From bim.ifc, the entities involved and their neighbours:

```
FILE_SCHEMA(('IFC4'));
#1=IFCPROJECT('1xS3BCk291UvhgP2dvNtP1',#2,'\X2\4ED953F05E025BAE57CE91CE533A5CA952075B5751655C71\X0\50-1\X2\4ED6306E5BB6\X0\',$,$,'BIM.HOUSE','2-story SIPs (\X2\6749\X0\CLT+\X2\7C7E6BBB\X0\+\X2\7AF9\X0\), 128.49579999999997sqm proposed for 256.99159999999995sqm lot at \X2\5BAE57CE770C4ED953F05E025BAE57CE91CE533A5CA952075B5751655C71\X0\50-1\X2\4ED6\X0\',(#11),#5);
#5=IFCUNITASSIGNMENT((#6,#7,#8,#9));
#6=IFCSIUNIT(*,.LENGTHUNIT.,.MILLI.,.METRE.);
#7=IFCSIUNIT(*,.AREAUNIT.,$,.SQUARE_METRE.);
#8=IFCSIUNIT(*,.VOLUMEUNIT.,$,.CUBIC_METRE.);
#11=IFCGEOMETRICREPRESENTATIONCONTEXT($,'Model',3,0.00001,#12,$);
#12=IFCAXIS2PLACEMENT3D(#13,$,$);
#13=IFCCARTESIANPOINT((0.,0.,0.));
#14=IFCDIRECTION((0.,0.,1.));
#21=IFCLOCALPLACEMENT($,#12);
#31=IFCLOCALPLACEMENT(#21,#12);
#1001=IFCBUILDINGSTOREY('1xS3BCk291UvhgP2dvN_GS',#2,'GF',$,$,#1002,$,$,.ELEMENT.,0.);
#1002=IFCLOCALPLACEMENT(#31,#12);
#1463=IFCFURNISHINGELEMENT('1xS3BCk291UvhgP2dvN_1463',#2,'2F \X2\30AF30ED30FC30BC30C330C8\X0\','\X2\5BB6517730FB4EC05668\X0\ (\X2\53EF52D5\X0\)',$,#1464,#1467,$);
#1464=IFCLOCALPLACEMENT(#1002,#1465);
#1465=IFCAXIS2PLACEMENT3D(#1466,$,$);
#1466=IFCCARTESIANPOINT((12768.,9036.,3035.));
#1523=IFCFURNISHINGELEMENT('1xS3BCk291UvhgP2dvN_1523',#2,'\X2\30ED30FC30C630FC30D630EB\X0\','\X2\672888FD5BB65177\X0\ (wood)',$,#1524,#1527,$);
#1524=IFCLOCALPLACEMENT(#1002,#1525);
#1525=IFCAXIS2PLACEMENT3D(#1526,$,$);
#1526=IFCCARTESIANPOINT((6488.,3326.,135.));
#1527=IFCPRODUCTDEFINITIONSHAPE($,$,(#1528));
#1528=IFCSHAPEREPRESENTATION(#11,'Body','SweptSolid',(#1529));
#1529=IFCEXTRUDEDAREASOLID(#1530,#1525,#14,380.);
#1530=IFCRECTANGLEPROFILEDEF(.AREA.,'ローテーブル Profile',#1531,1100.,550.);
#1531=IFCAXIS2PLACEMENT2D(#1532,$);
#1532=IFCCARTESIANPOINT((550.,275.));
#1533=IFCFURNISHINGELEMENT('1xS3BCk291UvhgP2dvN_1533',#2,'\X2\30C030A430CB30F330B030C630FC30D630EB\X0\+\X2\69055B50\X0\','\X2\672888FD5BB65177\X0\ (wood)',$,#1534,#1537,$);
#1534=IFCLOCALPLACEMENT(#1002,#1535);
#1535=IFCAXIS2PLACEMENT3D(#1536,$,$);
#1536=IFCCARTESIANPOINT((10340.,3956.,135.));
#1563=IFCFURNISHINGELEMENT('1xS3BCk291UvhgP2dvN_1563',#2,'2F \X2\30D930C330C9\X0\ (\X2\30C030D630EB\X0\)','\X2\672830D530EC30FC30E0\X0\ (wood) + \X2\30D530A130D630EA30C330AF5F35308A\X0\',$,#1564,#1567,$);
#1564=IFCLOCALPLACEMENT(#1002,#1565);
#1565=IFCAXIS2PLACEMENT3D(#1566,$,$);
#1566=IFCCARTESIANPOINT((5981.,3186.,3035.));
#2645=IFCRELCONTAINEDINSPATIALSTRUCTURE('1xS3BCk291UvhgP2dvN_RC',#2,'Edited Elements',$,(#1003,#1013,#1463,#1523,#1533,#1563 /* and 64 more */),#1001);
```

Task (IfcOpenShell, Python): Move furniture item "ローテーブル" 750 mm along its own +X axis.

```python
import ifcopenshell
import ifcopenshell.api.geometry
import ifcopenshell.util.placement
import ifcopenshell.util.unit

model = ifcopenshell.open("bim.ifc")
unit_scale = ifcopenshell.util.unit.calculate_unit_scale(model)

item = model.by_guid("1xS3BCk291UvhgP2dvN_1523")
matrix = ifcopenshell.util.placement.get_local_placement(item.ObjectPlacement)
matrix[:3, 3] += matrix[:3, 0] * 0.75 / unit_scale
ifcopenshell.api.geometry.edit_object_placement(model, product=item, matrix=matrix, is_si=False)

print(ifcopenshell.util.placement.get_local_placement(item.ObjectPlacement).round(3) + 0.0)

model.write("bim-out.ifc")
```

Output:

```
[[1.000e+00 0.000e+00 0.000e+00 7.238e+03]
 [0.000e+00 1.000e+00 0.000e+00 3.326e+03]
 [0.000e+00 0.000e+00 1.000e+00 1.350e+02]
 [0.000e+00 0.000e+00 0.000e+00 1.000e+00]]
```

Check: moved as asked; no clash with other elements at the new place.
